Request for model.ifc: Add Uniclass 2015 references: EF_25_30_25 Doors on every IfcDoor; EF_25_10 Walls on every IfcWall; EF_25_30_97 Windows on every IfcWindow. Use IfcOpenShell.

First a look at what the model holds.

```python
import ifcopenshell

model = ifcopenshell.open("model.ifc")
print(model.schema)
print("classifications:", [c.Name for c in model.by_type("IfcClassification")])
for ifc_class in ("IfcDoor", "IfcRoof", "IfcStair", "IfcWall", "IfcWindow"):
    print(ifc_class, len(model.by_type(ifc_class)))
```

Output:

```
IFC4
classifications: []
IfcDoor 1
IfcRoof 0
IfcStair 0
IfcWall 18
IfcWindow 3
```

```python
import ifcopenshell
import ifcopenshell.api.classification

model = ifcopenshell.open("model.ifc")

system = ifcopenshell.api.classification.add_classification(model, classification="Uniclass 2015")

codes = {
    "IfcDoor": ("EF_25_30_25", "Doors"),
    "IfcWall": ("EF_25_10", "Walls"),
    "IfcWindow": ("EF_25_30_97", "Windows"),
}
for ifc_class, (code, name) in codes.items():
    products = model.by_type(ifc_class)
    ifcopenshell.api.classification.add_reference(
        model, products=products, classification=system, identification=code, name=name
    )
    print(code, len(products))

model.write("model_edited.ifc")
```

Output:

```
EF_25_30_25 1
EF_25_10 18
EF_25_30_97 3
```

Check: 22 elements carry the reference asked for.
